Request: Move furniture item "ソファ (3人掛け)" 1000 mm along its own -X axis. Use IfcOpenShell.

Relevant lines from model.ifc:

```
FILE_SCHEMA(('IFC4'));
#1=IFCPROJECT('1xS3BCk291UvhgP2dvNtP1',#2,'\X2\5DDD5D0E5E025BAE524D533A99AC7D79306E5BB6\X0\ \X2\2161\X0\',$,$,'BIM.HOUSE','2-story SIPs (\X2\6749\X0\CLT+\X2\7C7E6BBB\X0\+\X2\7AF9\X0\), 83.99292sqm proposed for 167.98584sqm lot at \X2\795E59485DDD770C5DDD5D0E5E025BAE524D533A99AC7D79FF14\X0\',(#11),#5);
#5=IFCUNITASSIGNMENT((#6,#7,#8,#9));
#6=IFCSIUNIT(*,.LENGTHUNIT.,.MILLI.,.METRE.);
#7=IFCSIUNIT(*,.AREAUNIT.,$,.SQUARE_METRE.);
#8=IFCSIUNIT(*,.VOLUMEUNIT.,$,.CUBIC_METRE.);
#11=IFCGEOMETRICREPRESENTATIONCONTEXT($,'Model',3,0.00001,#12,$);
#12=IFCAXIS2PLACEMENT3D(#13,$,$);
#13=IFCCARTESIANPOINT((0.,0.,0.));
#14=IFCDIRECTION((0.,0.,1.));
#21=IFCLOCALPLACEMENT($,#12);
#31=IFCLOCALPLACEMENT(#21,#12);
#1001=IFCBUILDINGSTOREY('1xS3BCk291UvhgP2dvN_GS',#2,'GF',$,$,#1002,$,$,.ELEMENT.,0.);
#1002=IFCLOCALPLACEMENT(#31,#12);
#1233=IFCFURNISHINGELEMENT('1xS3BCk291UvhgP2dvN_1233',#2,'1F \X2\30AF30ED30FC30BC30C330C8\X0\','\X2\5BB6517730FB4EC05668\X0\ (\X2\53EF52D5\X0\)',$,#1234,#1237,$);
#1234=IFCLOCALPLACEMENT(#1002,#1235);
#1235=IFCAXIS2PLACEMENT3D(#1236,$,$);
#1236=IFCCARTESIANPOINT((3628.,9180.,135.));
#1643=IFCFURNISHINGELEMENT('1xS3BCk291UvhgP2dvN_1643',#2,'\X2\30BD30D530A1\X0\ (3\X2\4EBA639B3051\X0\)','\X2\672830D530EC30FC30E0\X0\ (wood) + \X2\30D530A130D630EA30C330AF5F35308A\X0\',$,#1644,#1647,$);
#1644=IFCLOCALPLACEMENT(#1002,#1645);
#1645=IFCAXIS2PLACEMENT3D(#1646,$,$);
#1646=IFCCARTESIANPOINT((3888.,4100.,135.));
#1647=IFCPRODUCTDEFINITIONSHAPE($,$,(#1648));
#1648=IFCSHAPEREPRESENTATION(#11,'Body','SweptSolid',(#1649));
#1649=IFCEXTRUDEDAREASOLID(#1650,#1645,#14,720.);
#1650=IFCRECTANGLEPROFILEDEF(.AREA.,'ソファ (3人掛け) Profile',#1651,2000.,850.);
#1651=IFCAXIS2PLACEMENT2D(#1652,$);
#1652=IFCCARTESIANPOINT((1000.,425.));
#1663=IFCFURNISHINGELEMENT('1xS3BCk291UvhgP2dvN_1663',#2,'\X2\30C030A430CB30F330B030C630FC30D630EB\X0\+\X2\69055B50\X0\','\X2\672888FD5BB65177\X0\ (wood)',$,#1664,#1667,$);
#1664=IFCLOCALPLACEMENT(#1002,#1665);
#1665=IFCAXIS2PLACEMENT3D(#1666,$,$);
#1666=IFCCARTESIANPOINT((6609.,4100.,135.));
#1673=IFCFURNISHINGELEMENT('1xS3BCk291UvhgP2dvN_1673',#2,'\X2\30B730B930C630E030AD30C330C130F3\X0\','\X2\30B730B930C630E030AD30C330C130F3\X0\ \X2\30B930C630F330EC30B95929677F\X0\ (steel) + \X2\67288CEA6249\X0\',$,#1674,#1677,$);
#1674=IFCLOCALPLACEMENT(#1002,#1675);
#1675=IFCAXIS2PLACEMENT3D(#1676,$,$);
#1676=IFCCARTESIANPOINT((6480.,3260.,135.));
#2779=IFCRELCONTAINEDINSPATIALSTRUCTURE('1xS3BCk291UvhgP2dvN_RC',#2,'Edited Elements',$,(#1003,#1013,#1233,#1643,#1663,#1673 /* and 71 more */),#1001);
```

```python
import ifcopenshell
import ifcopenshell.api.geometry
import ifcopenshell.util.placement

model = ifcopenshell.open("model.ifc")

item = model.by_id(1643)
matrix = ifcopenshell.util.placement.get_local_placement(item.ObjectPlacement)
matrix[:3, 3] -= matrix[:3, 0] * 1000.0
ifcopenshell.api.geometry.edit_object_placement(model, product=item, matrix=matrix, is_si=False)

print(ifcopenshell.util.placement.get_local_placement(item.ObjectPlacement).round(3) + 0.0)

model.write("model_rev.ifc")
```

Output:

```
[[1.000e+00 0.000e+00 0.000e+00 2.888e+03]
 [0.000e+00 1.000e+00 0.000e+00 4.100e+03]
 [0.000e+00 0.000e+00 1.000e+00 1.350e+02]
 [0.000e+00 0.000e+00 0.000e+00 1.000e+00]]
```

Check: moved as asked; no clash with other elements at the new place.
